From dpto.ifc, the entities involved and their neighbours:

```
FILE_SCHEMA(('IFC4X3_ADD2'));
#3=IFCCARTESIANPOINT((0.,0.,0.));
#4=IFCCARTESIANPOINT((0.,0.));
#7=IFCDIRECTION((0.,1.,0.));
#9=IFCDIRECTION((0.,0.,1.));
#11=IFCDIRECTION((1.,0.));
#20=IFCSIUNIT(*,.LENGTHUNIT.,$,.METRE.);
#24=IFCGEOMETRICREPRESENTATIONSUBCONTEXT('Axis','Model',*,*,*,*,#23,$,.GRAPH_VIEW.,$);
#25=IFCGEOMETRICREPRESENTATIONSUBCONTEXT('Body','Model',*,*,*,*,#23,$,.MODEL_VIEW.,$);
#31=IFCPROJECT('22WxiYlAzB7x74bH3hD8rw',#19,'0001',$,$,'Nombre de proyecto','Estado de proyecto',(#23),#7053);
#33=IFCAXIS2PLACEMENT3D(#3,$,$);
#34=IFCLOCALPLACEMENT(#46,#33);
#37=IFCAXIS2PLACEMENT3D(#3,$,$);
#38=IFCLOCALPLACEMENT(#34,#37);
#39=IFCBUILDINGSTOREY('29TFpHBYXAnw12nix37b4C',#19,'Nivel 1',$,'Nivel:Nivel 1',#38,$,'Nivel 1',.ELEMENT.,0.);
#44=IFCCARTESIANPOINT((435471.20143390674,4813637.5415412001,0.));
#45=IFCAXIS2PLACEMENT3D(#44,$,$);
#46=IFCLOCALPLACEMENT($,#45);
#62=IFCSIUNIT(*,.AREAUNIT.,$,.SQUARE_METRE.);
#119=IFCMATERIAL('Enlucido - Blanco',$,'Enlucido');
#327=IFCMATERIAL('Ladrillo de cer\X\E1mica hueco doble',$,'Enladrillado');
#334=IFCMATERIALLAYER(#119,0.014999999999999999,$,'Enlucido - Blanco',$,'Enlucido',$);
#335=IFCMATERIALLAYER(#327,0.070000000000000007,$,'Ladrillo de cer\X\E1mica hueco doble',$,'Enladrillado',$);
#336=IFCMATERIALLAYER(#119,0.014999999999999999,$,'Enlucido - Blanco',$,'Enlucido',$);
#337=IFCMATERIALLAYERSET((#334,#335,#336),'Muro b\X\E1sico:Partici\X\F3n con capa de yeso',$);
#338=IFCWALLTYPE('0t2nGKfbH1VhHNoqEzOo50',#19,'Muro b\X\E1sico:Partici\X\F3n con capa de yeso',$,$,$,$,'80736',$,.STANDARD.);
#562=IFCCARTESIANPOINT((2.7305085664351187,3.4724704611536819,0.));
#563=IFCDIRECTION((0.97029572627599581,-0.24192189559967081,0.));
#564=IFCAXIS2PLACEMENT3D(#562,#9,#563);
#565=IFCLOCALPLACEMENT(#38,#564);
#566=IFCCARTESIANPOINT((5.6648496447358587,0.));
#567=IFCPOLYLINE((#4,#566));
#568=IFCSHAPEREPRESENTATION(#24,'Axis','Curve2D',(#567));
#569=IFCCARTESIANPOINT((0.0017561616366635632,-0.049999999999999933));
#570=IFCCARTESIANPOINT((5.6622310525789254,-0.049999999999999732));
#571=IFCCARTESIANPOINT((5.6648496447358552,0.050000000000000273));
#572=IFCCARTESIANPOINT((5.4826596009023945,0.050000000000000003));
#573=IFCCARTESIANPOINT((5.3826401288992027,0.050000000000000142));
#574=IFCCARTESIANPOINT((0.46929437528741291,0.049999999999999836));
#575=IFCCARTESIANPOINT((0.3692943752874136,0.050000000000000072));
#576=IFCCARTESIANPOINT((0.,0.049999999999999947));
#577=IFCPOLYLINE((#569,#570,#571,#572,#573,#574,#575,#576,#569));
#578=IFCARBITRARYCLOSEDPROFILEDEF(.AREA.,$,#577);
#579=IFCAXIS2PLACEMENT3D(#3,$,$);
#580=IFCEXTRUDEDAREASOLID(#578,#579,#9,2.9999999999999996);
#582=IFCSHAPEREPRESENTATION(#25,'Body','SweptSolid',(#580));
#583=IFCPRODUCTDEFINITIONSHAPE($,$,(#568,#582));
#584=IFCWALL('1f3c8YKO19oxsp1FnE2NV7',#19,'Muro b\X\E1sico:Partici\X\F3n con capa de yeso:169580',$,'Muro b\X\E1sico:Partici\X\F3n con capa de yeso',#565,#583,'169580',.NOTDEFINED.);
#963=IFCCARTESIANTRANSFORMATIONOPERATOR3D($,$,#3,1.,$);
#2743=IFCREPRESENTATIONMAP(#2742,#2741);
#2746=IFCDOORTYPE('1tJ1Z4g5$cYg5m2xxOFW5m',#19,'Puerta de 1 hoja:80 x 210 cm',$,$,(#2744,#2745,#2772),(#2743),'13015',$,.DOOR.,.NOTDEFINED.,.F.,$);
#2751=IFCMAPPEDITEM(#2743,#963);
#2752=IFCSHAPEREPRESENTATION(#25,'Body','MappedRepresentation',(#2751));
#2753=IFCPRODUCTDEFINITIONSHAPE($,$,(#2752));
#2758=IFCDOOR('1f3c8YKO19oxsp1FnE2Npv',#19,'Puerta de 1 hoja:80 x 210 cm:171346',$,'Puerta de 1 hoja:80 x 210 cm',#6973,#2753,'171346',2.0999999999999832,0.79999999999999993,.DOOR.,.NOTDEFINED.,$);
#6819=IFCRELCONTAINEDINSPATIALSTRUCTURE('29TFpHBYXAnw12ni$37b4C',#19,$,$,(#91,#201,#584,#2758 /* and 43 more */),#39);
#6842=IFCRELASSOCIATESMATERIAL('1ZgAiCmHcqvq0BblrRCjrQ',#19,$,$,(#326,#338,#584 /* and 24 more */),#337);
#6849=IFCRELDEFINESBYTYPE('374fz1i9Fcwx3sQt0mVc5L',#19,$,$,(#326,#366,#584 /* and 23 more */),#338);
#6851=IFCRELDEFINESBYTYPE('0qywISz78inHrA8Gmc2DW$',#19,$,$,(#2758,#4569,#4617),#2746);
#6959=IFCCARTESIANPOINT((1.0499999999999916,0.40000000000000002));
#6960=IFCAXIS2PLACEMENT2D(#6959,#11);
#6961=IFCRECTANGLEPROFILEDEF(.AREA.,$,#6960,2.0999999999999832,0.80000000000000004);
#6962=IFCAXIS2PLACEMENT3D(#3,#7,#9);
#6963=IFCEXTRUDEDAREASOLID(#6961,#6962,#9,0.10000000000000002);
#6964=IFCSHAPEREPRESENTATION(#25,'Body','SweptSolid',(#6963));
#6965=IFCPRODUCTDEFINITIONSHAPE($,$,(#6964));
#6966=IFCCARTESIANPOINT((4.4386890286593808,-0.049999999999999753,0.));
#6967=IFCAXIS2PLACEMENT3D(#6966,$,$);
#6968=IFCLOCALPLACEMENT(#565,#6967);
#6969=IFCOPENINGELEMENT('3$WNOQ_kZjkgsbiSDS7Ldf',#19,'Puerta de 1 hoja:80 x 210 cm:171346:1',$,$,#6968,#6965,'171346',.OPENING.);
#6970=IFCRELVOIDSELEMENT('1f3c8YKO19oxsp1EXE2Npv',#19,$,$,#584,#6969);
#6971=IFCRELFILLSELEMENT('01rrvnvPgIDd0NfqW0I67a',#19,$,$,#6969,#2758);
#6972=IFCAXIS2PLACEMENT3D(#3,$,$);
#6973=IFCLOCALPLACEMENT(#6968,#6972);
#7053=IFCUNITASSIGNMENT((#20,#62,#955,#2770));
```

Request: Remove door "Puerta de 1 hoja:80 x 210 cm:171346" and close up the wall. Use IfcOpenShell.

```python
import ifcopenshell
import ifcopenshell.api.feature
import ifcopenshell.api.root
import ifcopenshell.geom
import ifcopenshell.util.shape

model = ifcopenshell.open("dpto.ifc")
settings = ifcopenshell.geom.settings()


def volume(element):
    """Net volume in cubic metres, openings subtracted."""
    shape = ifcopenshell.geom.create_shape(settings, element)
    return ifcopenshell.util.shape.get_volume(shape.geometry)


door = model.by_guid("1f3c8YKO19oxsp1FnE2Npv")
opening = door.FillsVoids[0].RelatingOpeningElement
wall = opening.VoidsElements[0].RelatingBuildingElement
before = volume(wall)

ifcopenshell.api.root.remove_product(model, product=door)
ifcopenshell.api.feature.remove_feature(model, feature=opening)

after = volume(wall)

print(f"wall volume {before:.3f} -> {after:.3f} m3")

model.write("dpto_v2.ifc")
```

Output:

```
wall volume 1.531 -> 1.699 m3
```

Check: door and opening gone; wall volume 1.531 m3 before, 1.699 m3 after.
